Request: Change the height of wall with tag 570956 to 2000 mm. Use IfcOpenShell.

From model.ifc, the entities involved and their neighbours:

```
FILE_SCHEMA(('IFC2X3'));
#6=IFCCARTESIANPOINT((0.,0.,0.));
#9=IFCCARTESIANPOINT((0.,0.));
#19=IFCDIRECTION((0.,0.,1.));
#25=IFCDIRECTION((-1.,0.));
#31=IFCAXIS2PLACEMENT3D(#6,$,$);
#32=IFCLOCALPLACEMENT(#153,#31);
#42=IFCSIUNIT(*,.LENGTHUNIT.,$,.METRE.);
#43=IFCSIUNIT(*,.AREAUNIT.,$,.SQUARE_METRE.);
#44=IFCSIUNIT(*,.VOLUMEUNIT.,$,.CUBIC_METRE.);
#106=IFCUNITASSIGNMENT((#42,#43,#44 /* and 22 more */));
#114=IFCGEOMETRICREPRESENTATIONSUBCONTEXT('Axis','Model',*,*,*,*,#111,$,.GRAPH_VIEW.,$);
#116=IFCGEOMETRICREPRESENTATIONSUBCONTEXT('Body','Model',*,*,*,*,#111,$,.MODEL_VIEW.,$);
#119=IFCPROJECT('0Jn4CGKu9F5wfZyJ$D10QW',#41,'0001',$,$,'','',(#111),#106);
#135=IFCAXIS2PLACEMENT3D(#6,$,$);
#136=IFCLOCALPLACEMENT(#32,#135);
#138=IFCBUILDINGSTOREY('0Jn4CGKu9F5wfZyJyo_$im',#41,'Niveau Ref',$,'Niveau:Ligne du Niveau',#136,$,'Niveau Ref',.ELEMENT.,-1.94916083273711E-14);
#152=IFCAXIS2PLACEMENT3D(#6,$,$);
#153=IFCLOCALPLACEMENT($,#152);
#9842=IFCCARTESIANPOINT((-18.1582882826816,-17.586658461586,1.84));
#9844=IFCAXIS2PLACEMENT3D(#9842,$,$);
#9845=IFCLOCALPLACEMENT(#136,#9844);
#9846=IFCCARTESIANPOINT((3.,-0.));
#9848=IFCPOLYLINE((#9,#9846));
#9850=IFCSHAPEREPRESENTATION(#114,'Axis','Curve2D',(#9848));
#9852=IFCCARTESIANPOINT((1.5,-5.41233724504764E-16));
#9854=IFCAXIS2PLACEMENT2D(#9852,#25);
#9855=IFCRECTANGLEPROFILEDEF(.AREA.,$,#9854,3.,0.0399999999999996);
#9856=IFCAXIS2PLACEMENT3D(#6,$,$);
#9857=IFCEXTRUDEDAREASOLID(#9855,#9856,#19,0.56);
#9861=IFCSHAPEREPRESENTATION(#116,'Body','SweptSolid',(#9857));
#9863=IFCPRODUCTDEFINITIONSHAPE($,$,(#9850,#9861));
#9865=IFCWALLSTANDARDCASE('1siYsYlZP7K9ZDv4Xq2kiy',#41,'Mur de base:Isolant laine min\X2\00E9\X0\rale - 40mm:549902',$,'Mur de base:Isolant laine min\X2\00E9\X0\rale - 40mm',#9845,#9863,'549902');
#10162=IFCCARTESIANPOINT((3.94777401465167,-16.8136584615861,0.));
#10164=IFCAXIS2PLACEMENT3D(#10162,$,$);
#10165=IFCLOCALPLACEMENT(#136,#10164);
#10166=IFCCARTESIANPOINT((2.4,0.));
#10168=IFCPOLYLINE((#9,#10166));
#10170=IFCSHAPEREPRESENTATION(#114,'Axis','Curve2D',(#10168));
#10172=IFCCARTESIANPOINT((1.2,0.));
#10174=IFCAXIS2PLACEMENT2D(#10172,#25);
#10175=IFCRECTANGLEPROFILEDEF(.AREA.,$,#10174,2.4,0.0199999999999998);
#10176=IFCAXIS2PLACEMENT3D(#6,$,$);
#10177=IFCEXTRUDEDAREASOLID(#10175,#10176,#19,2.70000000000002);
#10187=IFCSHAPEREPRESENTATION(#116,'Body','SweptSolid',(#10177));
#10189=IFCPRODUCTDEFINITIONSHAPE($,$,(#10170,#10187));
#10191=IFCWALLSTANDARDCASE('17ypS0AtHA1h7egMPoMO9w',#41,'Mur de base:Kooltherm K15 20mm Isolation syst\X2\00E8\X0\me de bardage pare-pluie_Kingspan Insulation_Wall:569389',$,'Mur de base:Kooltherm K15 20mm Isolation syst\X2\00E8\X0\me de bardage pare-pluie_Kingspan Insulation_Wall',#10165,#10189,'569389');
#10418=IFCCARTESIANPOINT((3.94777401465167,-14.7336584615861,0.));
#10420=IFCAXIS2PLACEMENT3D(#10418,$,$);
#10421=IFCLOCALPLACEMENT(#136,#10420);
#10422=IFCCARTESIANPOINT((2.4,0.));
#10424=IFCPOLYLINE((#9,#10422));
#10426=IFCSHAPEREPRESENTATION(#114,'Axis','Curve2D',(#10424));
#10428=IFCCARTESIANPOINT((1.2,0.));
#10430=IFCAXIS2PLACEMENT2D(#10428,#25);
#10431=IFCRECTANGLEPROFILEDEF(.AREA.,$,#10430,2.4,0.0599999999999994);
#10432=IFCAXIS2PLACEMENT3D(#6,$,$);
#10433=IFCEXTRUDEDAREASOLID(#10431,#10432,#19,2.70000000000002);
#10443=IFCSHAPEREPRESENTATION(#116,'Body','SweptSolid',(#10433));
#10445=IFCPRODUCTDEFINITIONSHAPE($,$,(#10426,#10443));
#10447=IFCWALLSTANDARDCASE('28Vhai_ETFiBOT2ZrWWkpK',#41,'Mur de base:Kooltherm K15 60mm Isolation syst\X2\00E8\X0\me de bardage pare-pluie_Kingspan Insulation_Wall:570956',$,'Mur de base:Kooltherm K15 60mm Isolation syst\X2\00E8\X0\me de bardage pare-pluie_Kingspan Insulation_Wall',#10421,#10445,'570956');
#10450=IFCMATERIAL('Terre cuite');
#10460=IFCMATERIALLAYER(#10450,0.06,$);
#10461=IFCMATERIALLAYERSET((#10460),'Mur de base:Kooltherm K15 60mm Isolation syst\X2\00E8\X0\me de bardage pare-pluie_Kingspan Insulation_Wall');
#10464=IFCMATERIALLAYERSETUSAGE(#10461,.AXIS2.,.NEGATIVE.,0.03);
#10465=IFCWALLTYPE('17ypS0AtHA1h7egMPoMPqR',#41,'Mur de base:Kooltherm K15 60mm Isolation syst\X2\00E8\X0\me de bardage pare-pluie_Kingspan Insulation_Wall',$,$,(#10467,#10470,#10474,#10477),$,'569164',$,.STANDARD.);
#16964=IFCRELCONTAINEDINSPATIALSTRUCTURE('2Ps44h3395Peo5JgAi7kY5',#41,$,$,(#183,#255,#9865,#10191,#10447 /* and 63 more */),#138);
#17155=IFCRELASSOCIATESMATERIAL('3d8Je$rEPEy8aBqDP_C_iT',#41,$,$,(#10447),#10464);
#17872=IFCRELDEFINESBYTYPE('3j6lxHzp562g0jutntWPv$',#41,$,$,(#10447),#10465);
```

```python
import ifcopenshell
import ifcopenshell.geom
import ifcopenshell.util.representation
import ifcopenshell.util.shape
import ifcopenshell.util.unit

model = ifcopenshell.open("model.ifc")
unit_scale = ifcopenshell.util.unit.calculate_unit_scale(model)
settings = ifcopenshell.geom.settings()


def volume(element):
    """Net volume in cubic metres, openings subtracted."""
    shape = ifcopenshell.geom.create_shape(settings, element)
    return ifcopenshell.util.shape.get_volume(shape.geometry)


wall = model.by_id(10447)
before = volume(wall)

body = ifcopenshell.util.representation.get_representation(wall, "Model", "Body")
solid = body.Items[0]
old_height = solid.Depth
solid.Depth = 2 / unit_scale
after = volume(wall)

print(f"height {old_height:g} -> {solid.Depth:g}, volume {before:.3f} -> {after:.3f} m3")

model.write("model_rev.ifc")
```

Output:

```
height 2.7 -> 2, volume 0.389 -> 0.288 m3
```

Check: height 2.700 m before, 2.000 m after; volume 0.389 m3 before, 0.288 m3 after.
